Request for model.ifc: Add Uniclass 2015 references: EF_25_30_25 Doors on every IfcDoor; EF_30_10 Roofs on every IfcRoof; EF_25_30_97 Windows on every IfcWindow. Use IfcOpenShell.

First a look at what the model holds.

```python
import ifcopenshell

model = ifcopenshell.open("model.ifc")
print(model.schema)
print("classifications:", [c.Name for c in model.by_type("IfcClassification")])
for ifc_class in ("IfcDoor", "IfcRoof", "IfcStair", "IfcWall", "IfcWindow"):
    print(ifc_class, len(model.by_type(ifc_class)))
```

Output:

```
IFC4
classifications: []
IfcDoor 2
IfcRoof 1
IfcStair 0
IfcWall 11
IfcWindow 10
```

```python
import ifcopenshell
import ifcopenshell.api.classification

model = ifcopenshell.open("model.ifc")

system = ifcopenshell.api.classification.add_classification(model, classification="Uniclass 2015")

codes = {
    "IfcDoor": ("EF_25_30_25", "Doors"),
    "IfcRoof": ("EF_30_10", "Roofs"),
    "IfcWindow": ("EF_25_30_97", "Windows"),
}
for ifc_class, (code, name) in codes.items():
    products = model.by_type(ifc_class)
    ifcopenshell.api.classification.add_reference(
        model, products=products, classification=system, identification=code, name=name
    )
    print(code, len(products))

model.write("model-out.ifc")
```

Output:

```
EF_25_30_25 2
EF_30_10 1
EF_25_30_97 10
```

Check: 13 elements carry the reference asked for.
